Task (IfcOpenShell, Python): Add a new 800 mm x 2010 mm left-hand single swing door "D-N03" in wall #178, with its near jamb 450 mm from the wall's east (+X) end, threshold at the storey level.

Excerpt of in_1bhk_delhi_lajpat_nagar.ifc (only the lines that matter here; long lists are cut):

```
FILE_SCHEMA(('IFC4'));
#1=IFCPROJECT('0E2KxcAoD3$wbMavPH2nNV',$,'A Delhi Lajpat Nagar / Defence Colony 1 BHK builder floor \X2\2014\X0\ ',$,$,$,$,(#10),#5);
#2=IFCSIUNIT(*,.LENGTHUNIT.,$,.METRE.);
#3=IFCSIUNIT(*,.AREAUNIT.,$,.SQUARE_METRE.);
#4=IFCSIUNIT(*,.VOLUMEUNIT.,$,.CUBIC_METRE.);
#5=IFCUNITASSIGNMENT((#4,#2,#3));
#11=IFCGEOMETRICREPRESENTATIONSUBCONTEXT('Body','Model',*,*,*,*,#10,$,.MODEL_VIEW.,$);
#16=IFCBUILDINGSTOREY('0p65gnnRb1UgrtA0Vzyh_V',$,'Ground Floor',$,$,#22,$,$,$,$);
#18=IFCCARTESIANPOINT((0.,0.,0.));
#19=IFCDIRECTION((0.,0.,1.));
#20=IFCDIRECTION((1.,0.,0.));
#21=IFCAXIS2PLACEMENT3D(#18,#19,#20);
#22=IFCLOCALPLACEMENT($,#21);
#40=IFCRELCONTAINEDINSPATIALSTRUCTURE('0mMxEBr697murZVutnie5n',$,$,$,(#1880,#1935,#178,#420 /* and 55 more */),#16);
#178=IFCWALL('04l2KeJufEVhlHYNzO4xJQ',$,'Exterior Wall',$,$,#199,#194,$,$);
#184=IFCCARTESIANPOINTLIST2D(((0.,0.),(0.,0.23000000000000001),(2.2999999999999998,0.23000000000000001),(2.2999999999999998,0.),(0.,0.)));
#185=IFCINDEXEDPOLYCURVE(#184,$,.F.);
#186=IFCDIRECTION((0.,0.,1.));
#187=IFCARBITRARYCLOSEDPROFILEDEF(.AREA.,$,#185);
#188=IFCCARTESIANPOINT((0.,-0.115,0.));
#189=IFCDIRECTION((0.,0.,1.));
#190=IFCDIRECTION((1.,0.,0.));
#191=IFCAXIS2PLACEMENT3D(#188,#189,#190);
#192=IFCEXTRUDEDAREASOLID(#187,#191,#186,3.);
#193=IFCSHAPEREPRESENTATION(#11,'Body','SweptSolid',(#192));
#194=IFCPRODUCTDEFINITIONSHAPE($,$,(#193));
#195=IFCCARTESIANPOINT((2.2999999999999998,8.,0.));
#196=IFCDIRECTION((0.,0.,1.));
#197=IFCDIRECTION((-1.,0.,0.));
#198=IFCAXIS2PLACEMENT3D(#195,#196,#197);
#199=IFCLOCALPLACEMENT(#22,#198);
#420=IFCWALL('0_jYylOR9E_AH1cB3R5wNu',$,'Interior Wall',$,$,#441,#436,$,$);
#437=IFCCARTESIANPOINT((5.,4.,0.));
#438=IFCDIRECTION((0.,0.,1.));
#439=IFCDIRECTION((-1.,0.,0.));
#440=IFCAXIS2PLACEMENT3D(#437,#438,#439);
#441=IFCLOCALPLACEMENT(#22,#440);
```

```python
import numpy as np
import ifcopenshell
import ifcopenshell.api.feature
import ifcopenshell.api.geometry
import ifcopenshell.api.root
import ifcopenshell.api.spatial
import ifcopenshell.geom
import ifcopenshell.util.element
import ifcopenshell.util.placement
import ifcopenshell.util.representation
import ifcopenshell.util.shape
import ifcopenshell.util.unit

model = ifcopenshell.open("in_1bhk_delhi_lajpat_nagar.ifc")
unit_scale = ifcopenshell.util.unit.calculate_unit_scale(model)
settings = ifcopenshell.geom.settings()


def volume(element):
    """Net volume in cubic metres, openings subtracted."""
    shape = ifcopenshell.geom.create_shape(settings, element)
    return ifcopenshell.util.shape.get_volume(shape.geometry)


wall = model.by_guid("04l2KeJufEVhlHYNzO4xJQ")
storey = ifcopenshell.util.element.get_container(wall, ifc_class="IfcBuildingStorey")
context = ifcopenshell.util.representation.get_context(model, "Model", "Body", "MODEL_VIEW")
before = volume(wall)

width, height, from_end, sill = 0.8, 2.01, 0.45, 0.0  # metres

# The wall runs along its own X axis, and the end named is its -X end.
wall_shape = ifcopenshell.geom.create_shape(settings, wall)
x, y, z = ifcopenshell.util.shape.get_vertices(wall_shape.geometry).T
start = x.min() + from_end
face, thickness = float(y.min()), float(y.max() - y.min())
wall_matrix = ifcopenshell.util.placement.get_local_placement(wall.ObjectPlacement)
level = ifcopenshell.util.placement.get_local_placement(storey.ObjectPlacement)[2, 3]


def in_wall(x, y):
    """Placement at x, y metres in the wall's axes, at sill height."""
    matrix = wall_matrix.copy()
    matrix[:, 3] = wall_matrix @ np.array([x / unit_scale, y / unit_scale, 0.0, 1.0])
    matrix[2, 3] = level + sill / unit_scale
    return matrix


# Opening: a box that overshoots both wall faces by 50 mm.
opening = ifcopenshell.api.root.create_entity(model, ifc_class="IfcOpeningElement", predefined_type="OPENING")
box = ifcopenshell.api.geometry.add_wall_representation(
    model, context=context, length=width, height=height, thickness=thickness + 0.1
)
ifcopenshell.api.geometry.assign_representation(model, product=opening, representation=box)
ifcopenshell.api.geometry.edit_object_placement(model, product=opening, matrix=in_wall(start, face - 0.05), is_si=False)
ifcopenshell.api.feature.add_feature(model, feature=opening, element=wall)

door = ifcopenshell.api.root.create_entity(model, ifc_class="IfcDoor", name="D-N03", predefined_type="DOOR")
door.OverallWidth, door.OverallHeight = width / unit_scale, height / unit_scale
door.OperationType = "SINGLE_SWING_LEFT"
body = ifcopenshell.api.geometry.add_door_representation(
    model,
    context=context,
    overall_width=door.OverallWidth,
    overall_height=door.OverallHeight,
    operation_type="SINGLE_SWING_LEFT",
    lining_properties={"LiningDepth": thickness / unit_scale, "ThresholdDepth": thickness / unit_scale},
)
ifcopenshell.api.geometry.assign_representation(model, product=door, representation=body)
ifcopenshell.api.spatial.assign_container(model, products=[door], relating_structure=storey)
ifcopenshell.api.feature.add_filling(model, opening=opening, element=door)

# The lining spans the wall, so the door starts at the wall face.
ifcopenshell.api.geometry.edit_object_placement(model, product=door, matrix=in_wall(start, face), is_si=False)

after = volume(wall)

print(f"wall volume {before:.3f} -> {after:.3f} m3")

model.write("in_1bhk_delhi_lajpat_nagar-out.ifc")
```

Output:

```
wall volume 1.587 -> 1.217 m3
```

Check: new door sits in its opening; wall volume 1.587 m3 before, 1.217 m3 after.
